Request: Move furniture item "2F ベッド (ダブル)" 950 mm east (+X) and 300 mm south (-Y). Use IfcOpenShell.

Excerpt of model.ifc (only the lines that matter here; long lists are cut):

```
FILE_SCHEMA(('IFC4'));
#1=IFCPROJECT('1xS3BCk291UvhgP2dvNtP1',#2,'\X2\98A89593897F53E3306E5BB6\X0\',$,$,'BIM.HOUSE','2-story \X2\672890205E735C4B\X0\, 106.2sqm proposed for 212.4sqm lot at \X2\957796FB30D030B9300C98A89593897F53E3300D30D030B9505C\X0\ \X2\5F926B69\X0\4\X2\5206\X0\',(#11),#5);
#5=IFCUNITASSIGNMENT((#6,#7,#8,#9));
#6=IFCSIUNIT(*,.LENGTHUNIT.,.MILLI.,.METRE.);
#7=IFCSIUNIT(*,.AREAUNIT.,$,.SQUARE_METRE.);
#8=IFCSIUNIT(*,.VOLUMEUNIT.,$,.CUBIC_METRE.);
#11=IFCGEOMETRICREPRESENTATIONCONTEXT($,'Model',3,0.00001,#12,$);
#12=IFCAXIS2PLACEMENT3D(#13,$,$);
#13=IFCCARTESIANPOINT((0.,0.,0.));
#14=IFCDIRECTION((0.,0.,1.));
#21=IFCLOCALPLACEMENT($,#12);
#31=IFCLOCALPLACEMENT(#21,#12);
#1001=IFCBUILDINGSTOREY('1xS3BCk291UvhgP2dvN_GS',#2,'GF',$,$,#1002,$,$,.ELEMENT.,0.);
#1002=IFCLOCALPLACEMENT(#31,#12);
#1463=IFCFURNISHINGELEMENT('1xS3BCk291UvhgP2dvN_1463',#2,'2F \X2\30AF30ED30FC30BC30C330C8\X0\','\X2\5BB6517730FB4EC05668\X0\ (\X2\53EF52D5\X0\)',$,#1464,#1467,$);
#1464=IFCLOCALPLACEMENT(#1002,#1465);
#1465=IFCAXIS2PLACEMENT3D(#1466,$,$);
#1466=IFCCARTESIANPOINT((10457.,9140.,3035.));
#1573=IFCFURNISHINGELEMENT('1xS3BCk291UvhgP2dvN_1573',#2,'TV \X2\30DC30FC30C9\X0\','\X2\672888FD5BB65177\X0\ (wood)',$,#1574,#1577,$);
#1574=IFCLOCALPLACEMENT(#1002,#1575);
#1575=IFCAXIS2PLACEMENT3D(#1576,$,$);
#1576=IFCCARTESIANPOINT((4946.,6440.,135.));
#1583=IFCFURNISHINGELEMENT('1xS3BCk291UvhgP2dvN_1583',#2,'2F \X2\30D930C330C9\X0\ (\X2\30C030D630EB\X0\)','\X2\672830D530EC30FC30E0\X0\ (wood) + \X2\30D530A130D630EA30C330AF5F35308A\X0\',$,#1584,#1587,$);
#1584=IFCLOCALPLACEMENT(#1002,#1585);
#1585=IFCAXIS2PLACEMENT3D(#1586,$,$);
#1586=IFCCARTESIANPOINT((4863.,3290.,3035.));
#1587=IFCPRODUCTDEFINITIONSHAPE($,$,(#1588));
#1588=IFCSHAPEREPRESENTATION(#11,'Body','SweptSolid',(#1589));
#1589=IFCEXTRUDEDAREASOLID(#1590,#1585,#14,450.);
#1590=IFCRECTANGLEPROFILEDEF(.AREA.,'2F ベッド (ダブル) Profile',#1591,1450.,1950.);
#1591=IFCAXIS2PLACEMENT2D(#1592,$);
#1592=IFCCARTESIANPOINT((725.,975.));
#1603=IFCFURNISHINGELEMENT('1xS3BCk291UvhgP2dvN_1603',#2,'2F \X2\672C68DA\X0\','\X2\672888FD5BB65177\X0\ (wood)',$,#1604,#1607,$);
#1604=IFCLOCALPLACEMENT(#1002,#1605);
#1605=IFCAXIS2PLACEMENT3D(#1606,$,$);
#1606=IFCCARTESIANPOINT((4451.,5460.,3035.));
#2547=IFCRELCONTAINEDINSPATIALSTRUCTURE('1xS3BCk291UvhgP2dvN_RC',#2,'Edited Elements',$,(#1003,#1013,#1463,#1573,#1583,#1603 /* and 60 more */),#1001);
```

```python
import ifcopenshell
import ifcopenshell.api.geometry
import ifcopenshell.util.placement

model = ifcopenshell.open("model.ifc")

item = model.by_guid("1xS3BCk291UvhgP2dvN_1583")
matrix = ifcopenshell.util.placement.get_local_placement(item.ObjectPlacement)
matrix[0, 3] += 950.0
matrix[1, 3] -= 300.0
ifcopenshell.api.geometry.edit_object_placement(model, product=item, matrix=matrix, is_si=False)

print(ifcopenshell.util.placement.get_local_placement(item.ObjectPlacement).round(3) + 0.0)

model.write("model_rev.ifc")
```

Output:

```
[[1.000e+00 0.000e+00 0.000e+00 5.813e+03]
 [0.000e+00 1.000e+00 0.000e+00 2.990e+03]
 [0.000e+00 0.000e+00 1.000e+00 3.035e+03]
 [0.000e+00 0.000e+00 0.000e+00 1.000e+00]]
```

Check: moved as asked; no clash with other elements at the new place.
